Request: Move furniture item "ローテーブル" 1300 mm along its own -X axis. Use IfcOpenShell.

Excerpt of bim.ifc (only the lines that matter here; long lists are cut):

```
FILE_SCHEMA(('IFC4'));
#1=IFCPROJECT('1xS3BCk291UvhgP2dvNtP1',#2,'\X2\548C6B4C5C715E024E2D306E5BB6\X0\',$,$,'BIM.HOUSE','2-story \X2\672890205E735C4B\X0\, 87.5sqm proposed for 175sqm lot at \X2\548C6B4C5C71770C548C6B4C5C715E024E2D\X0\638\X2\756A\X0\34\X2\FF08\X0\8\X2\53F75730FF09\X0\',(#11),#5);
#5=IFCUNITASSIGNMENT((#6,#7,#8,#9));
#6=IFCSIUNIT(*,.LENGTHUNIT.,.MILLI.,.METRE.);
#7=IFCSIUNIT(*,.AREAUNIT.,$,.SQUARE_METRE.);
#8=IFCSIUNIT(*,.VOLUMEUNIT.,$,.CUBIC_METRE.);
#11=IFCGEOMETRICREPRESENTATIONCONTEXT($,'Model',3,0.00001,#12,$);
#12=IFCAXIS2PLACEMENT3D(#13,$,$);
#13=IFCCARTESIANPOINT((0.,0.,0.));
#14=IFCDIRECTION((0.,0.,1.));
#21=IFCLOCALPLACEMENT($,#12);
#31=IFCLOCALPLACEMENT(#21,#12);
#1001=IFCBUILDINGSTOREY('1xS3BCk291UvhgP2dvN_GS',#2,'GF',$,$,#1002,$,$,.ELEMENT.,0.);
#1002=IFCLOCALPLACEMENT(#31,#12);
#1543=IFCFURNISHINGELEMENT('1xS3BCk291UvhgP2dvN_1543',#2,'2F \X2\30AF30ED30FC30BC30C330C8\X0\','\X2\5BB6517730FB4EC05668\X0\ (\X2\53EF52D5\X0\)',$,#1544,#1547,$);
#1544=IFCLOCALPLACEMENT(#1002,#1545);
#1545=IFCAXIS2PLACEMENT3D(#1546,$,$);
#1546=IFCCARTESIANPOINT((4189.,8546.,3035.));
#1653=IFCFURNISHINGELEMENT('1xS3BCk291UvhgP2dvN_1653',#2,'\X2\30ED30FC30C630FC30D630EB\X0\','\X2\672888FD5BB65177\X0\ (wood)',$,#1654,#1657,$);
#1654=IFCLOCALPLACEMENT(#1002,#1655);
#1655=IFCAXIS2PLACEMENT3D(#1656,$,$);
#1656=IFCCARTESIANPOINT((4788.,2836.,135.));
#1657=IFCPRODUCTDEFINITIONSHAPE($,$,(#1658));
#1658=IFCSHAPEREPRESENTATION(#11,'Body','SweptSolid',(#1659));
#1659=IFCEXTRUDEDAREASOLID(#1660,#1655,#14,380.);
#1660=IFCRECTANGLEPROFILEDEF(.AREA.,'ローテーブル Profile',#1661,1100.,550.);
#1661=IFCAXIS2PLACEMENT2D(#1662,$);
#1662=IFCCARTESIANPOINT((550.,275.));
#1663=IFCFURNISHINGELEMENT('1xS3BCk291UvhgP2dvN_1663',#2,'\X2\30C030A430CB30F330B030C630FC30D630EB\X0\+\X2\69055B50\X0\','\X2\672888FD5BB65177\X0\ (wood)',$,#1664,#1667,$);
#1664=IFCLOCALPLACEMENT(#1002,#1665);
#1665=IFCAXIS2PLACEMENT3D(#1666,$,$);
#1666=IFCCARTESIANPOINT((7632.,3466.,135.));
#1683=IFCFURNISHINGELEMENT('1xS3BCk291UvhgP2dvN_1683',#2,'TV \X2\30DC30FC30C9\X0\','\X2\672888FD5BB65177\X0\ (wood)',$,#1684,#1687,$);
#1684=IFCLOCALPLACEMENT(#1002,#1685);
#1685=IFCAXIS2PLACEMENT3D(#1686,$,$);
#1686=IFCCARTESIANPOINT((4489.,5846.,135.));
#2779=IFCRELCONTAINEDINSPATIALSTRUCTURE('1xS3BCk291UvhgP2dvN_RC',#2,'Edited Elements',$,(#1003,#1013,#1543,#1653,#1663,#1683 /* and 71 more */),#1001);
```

```python
import ifcopenshell
import ifcopenshell.api.geometry
import ifcopenshell.util.placement

model = ifcopenshell.open("bim.ifc")

item = model.by_guid("1xS3BCk291UvhgP2dvN_1653")
matrix = ifcopenshell.util.placement.get_local_placement(item.ObjectPlacement)
matrix[:3, 3] -= matrix[:3, 0] * 1300.0
ifcopenshell.api.geometry.edit_object_placement(model, product=item, matrix=matrix, is_si=False)

print(ifcopenshell.util.placement.get_local_placement(item.ObjectPlacement).round(3) + 0.0)

model.write("bim_edited.ifc")
```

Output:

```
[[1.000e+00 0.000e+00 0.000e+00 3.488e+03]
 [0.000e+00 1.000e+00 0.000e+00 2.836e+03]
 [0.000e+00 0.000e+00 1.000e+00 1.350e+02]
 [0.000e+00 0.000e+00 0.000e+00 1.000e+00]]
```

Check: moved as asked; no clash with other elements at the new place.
